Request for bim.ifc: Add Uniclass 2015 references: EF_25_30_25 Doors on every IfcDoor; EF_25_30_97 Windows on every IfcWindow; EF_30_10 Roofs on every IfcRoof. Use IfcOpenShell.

First a look at what the model holds.

```python
import ifcopenshell

model = ifcopenshell.open("bim.ifc")
print(model.schema)
print("classifications:", [c.Name for c in model.by_type("IfcClassification")])
for ifc_class in ("IfcDoor", "IfcRoof", "IfcStair", "IfcWall", "IfcWindow"):
    print(ifc_class, len(model.by_type(ifc_class)))
```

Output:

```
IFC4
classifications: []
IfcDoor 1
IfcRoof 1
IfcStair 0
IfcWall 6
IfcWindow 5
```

```python
import ifcopenshell
import ifcopenshell.api.classification

model = ifcopenshell.open("bim.ifc")

system = ifcopenshell.api.classification.add_classification(model, classification="Uniclass 2015")

codes = {
    "IfcDoor": ("EF_25_30_25", "Doors"),
    "IfcWindow": ("EF_25_30_97", "Windows"),
    "IfcRoof": ("EF_30_10", "Roofs"),
}
for ifc_class, (code, name) in codes.items():
    products = model.by_type(ifc_class)
    ifcopenshell.api.classification.add_reference(
        model, products=products, classification=system, identification=code, name=name
    )
    print(code, len(products))

model.write("bim_rev.ifc")
```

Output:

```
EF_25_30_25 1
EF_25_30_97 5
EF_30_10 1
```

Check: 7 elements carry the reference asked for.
